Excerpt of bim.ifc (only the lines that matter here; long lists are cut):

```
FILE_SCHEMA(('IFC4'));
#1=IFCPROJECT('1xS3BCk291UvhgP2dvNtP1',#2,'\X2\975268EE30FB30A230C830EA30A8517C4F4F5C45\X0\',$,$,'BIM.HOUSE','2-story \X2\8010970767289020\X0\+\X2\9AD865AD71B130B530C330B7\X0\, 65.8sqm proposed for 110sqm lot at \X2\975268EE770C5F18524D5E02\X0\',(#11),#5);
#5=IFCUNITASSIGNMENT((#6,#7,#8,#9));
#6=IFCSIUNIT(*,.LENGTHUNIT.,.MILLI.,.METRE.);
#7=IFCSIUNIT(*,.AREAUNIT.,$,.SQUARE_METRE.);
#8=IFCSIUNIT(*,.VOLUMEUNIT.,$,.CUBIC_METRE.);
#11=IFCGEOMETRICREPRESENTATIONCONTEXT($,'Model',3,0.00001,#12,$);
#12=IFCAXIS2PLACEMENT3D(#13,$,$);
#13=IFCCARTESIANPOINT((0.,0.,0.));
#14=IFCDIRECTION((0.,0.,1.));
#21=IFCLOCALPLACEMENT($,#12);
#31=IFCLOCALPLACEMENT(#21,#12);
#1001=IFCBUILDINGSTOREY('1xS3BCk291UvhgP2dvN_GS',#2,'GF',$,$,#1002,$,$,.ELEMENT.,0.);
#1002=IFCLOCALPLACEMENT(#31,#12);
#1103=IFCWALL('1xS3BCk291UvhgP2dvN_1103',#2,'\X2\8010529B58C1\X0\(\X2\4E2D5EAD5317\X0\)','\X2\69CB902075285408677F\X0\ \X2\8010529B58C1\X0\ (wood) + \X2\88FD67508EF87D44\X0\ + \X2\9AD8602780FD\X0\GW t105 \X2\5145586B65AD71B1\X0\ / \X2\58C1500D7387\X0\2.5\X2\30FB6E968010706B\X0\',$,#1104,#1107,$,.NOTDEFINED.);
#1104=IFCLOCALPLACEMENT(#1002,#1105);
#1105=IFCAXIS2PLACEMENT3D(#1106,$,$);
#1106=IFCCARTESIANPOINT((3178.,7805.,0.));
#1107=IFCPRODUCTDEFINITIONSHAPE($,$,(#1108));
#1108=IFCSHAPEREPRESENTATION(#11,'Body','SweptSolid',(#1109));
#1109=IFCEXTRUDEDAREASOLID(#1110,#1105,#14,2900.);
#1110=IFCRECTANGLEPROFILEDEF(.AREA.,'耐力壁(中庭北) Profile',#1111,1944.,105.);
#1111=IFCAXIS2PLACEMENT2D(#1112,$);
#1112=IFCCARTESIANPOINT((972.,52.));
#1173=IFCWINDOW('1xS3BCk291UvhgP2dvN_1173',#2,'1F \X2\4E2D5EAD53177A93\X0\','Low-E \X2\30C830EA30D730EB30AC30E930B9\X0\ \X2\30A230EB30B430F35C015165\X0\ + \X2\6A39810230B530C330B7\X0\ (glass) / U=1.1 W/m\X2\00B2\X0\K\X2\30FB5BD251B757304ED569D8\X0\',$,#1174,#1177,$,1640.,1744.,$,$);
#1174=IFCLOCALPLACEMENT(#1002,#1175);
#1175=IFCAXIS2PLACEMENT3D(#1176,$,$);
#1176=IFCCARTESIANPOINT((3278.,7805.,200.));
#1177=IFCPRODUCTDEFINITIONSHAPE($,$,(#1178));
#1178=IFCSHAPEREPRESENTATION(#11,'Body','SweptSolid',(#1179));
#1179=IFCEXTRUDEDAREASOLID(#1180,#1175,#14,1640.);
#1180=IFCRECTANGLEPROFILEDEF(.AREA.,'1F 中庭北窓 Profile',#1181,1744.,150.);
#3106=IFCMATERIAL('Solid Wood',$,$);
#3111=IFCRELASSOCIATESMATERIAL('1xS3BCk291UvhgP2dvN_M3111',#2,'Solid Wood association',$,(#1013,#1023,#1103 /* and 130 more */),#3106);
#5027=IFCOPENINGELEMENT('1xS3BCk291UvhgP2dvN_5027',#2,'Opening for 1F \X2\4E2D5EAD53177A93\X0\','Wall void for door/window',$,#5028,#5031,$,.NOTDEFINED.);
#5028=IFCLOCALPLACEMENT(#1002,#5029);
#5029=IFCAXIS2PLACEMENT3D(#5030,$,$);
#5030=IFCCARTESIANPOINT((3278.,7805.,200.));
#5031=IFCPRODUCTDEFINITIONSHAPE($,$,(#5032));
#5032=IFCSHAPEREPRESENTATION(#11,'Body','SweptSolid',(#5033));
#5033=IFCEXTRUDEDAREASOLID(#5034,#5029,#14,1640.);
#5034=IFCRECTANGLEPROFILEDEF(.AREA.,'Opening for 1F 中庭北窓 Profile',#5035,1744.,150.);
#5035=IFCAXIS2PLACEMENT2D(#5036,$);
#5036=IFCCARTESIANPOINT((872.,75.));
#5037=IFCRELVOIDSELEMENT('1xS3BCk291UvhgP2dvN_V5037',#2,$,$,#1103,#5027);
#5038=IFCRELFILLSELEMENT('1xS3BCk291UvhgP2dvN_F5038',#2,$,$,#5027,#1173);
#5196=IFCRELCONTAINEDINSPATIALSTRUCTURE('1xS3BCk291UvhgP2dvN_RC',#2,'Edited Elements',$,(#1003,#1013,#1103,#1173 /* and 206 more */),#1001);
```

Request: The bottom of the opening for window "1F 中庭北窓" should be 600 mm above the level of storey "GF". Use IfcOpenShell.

```python
import numpy as np
import ifcopenshell
import ifcopenshell.api.geometry
import ifcopenshell.geom
import ifcopenshell.util.element
import ifcopenshell.util.placement
import ifcopenshell.util.shape
import ifcopenshell.util.unit

model = ifcopenshell.open("bim.ifc")
unit_scale = ifcopenshell.util.unit.calculate_unit_scale(model)

window = model.by_id(1173)
opening = window.FillsVoids[0].RelatingOpeningElement
storey = ifcopenshell.util.element.get_container(window, ifc_class="IfcBuildingStorey")
level = ifcopenshell.util.placement.get_local_placement(storey.ObjectPlacement)[2, 3]

# The opening's origin need not be at the sill, so measure its lowest point.
shape = ifcopenshell.geom.create_shape(ifcopenshell.geom.settings(), opening)
bottom = ifcopenshell.util.shape.get_shape_bottom_elevation(shape, shape.geometry) / unit_scale
dz = level + 600.0 - bottom

shift = np.array([0.0, 0.0, dz])
# The window is not placed relative to its opening, so move both.
for product in (opening, window):
    matrix = ifcopenshell.util.placement.get_local_placement(product.ObjectPlacement)
    matrix[:3, 3] += shift
    ifcopenshell.api.geometry.edit_object_placement(model, product=product, matrix=matrix, is_si=False)

print(f"moved by {dz * unit_scale:+.3f} m")

model.write("bim_updated.ifc")
```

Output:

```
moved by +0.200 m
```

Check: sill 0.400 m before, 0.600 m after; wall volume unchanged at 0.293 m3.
